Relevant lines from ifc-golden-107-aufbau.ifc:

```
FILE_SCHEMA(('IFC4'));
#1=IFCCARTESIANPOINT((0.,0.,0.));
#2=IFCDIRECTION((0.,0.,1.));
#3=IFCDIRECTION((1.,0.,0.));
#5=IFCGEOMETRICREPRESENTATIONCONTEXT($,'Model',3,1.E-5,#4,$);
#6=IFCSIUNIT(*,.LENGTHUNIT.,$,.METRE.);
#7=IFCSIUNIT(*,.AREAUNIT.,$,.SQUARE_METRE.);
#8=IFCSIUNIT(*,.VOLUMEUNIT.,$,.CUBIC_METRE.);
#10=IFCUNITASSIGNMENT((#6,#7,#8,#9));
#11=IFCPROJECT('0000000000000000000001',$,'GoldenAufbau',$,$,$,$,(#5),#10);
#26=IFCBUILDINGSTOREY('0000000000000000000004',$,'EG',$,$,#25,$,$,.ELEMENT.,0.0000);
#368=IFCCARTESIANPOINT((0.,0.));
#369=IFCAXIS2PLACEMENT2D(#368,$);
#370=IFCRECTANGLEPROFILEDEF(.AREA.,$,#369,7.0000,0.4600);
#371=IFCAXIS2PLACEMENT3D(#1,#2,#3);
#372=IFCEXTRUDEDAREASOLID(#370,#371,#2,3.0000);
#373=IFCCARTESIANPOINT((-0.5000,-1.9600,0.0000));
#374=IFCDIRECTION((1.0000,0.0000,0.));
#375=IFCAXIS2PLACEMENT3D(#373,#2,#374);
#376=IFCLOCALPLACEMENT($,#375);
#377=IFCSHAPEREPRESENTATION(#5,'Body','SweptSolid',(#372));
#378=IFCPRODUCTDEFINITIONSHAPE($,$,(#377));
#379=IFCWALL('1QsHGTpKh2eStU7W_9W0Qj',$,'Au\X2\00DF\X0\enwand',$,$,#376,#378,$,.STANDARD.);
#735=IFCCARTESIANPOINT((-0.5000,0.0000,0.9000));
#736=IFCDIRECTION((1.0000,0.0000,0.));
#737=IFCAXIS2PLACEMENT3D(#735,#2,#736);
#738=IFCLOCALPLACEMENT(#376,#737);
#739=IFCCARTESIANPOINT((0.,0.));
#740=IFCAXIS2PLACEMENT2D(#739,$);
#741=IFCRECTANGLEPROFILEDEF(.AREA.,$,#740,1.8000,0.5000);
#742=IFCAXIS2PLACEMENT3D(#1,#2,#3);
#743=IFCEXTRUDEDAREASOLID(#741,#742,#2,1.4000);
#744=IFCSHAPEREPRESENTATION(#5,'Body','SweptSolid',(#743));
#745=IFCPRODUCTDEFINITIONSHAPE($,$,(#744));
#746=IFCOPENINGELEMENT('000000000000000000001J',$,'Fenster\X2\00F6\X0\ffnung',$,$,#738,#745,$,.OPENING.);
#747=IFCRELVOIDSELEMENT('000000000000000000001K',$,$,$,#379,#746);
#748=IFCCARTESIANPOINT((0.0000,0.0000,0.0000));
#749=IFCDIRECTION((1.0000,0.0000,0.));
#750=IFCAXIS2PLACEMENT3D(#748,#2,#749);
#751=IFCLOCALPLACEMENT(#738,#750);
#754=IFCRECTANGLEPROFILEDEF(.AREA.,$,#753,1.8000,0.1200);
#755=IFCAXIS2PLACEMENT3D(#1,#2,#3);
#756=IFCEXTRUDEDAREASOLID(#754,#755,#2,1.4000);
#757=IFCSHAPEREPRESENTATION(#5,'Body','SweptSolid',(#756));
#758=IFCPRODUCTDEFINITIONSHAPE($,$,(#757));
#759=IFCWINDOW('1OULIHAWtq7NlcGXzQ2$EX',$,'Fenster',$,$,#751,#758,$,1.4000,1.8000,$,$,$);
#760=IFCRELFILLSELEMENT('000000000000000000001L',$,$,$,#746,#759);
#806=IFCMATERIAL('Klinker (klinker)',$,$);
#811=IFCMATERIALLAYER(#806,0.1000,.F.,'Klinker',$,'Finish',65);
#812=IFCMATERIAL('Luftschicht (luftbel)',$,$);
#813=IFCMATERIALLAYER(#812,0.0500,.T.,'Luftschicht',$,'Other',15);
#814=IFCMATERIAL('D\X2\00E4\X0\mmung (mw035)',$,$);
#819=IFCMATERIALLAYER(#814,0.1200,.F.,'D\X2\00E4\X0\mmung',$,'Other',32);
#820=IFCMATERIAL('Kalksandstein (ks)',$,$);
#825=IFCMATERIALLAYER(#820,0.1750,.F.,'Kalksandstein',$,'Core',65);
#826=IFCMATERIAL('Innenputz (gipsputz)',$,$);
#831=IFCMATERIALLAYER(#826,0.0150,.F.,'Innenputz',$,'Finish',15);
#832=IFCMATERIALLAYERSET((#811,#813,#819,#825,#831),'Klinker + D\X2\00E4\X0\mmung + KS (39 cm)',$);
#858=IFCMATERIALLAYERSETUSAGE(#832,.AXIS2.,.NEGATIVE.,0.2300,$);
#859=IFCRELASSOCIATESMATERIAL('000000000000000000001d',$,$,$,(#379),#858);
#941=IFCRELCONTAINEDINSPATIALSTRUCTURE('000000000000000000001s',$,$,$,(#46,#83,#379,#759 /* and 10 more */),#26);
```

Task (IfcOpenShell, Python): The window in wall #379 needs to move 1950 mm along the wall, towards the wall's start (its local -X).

```python
import ifcopenshell
import ifcopenshell.api.geometry
import ifcopenshell.util.placement
import ifcopenshell.util.unit

model = ifcopenshell.open("ifc-golden-107-aufbau.ifc")
unit_scale = ifcopenshell.util.unit.calculate_unit_scale(model)

window = model.by_id(759)
opening = window.FillsVoids[0].RelatingOpeningElement
wall = opening.VoidsElements[0].RelatingBuildingElement

wall_matrix = ifcopenshell.util.placement.get_local_placement(wall.ObjectPlacement)
shift = wall_matrix[:3, 0] * -1.95 / unit_scale
before = ifcopenshell.util.placement.get_local_placement(window.ObjectPlacement)[:3, 3].copy()

# The window is placed relative to its opening, so it follows when the opening moves.
matrix = ifcopenshell.util.placement.get_local_placement(opening.ObjectPlacement)
matrix[:3, 3] += shift
ifcopenshell.api.geometry.edit_object_placement(
    model, product=opening, matrix=matrix, is_si=False, should_transform_children=True
)

after = ifcopenshell.util.placement.get_local_placement(window.ObjectPlacement)[:3, 3]
print("window moved by", (after - before).round(3) + 0.0)

model.write("ifc-golden-107-aufbau_rev.ifc")
```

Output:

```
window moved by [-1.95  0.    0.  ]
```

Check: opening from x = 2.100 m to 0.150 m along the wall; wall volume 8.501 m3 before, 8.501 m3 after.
